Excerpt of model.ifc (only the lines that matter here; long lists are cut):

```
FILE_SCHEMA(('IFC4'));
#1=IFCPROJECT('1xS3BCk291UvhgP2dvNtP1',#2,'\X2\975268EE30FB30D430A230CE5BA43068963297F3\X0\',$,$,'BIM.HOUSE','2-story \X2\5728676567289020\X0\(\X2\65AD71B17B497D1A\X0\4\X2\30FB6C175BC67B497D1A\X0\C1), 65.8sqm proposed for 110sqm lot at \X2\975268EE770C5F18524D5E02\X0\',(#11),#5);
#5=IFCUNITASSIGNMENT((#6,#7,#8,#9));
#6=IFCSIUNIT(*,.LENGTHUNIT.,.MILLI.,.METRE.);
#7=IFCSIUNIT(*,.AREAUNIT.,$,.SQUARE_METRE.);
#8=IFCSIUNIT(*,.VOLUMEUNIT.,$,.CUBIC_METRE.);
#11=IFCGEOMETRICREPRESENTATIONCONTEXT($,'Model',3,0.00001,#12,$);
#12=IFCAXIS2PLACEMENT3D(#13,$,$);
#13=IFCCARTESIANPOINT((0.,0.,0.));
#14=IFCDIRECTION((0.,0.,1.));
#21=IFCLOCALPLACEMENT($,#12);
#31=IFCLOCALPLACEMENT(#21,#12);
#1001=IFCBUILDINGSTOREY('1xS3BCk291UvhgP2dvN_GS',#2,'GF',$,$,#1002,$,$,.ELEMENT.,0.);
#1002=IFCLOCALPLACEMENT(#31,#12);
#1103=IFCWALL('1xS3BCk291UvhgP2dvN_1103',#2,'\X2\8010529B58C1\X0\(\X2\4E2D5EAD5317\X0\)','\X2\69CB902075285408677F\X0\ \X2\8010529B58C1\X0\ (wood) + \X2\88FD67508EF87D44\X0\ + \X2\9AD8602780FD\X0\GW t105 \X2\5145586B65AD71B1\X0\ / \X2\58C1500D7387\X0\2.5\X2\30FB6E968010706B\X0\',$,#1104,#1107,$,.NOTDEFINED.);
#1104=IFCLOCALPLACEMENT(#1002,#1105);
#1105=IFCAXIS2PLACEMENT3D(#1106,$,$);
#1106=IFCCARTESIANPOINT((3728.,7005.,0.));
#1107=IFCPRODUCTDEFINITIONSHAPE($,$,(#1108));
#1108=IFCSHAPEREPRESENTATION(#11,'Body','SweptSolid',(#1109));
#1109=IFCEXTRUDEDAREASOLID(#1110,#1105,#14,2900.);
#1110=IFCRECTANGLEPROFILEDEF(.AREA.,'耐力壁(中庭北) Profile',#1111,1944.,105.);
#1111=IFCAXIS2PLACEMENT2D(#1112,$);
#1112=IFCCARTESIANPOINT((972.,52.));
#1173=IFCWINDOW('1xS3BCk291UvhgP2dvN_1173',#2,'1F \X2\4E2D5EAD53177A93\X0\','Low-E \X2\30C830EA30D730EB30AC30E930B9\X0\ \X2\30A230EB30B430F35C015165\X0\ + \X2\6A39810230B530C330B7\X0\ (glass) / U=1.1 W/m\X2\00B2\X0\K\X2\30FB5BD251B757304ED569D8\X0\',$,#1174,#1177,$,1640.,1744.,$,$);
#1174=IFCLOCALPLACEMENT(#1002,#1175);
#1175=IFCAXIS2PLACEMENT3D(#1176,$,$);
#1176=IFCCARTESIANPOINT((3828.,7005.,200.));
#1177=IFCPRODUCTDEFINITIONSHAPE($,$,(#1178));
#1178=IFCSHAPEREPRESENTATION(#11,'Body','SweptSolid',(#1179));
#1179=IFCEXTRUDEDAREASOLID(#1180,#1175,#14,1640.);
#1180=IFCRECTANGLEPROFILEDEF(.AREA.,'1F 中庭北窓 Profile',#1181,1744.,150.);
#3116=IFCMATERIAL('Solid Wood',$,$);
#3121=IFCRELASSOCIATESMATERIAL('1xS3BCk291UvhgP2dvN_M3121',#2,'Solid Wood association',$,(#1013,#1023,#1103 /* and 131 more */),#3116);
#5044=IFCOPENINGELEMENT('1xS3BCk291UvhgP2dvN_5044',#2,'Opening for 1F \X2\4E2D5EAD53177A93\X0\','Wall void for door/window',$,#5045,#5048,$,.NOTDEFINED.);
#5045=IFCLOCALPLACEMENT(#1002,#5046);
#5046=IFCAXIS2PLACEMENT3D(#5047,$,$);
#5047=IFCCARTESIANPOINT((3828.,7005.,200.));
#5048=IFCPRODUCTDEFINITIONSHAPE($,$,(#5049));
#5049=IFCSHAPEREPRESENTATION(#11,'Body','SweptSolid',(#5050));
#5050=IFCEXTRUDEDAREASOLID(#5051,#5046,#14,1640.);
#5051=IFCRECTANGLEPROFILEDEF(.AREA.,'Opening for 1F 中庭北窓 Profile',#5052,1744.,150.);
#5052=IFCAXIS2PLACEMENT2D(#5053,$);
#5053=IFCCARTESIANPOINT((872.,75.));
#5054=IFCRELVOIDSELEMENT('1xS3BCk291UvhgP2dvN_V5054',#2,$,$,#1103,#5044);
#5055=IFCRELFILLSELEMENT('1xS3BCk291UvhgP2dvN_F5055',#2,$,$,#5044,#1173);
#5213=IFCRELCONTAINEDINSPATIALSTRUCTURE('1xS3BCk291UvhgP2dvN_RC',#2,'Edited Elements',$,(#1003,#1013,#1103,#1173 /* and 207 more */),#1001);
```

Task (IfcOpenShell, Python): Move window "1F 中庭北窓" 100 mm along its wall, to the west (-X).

```python
import ifcopenshell
import ifcopenshell.api.geometry
import ifcopenshell.util.placement
import ifcopenshell.util.unit

model = ifcopenshell.open("model.ifc")
unit_scale = ifcopenshell.util.unit.calculate_unit_scale(model)

window = model.by_guid("1xS3BCk291UvhgP2dvN_1173")
opening = window.FillsVoids[0].RelatingOpeningElement
wall = opening.VoidsElements[0].RelatingBuildingElement

wall_matrix = ifcopenshell.util.placement.get_local_placement(wall.ObjectPlacement)
shift = wall_matrix[:3, 0] * -0.1 / unit_scale
before = ifcopenshell.util.placement.get_local_placement(window.ObjectPlacement)[:3, 3].copy()

# The window is not placed relative to its opening, so move both.
for product in (opening, window):
    matrix = ifcopenshell.util.placement.get_local_placement(product.ObjectPlacement)
    matrix[:3, 3] += shift
    ifcopenshell.api.geometry.edit_object_placement(model, product=product, matrix=matrix, is_si=False)

after = ifcopenshell.util.placement.get_local_placement(window.ObjectPlacement)[:3, 3]
print("window moved by", (after - before).round(3) + 0.0)

model.write("model_updated.ifc")
```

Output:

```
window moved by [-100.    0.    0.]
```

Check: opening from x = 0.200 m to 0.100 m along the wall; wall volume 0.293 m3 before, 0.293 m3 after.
